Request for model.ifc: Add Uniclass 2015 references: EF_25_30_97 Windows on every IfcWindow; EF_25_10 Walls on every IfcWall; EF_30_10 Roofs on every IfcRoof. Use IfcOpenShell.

First a look at what the model holds.

```python
import ifcopenshell

model = ifcopenshell.open("model.ifc")
print(model.schema)
print("classifications:", [c.Name for c in model.by_type("IfcClassification")])
for ifc_class in ("IfcDoor", "IfcRoof", "IfcStair", "IfcWall", "IfcWindow"):
    print(ifc_class, len(model.by_type(ifc_class)))
```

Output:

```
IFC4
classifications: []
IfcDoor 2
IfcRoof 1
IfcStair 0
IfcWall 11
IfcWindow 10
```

```python
import ifcopenshell
import ifcopenshell.api.classification

model = ifcopenshell.open("model.ifc")

system = ifcopenshell.api.classification.add_classification(model, classification="Uniclass 2015")

codes = {
    "IfcWindow": ("EF_25_30_97", "Windows"),
    "IfcWall": ("EF_25_10", "Walls"),
    "IfcRoof": ("EF_30_10", "Roofs"),
}
for ifc_class, (code, name) in codes.items():
    products = model.by_type(ifc_class)
    ifcopenshell.api.classification.add_reference(
        model, products=products, classification=system, identification=code, name=name
    )
    print(code, len(products))

model.write("model-out.ifc")
```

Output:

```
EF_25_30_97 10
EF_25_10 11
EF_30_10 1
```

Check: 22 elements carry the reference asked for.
